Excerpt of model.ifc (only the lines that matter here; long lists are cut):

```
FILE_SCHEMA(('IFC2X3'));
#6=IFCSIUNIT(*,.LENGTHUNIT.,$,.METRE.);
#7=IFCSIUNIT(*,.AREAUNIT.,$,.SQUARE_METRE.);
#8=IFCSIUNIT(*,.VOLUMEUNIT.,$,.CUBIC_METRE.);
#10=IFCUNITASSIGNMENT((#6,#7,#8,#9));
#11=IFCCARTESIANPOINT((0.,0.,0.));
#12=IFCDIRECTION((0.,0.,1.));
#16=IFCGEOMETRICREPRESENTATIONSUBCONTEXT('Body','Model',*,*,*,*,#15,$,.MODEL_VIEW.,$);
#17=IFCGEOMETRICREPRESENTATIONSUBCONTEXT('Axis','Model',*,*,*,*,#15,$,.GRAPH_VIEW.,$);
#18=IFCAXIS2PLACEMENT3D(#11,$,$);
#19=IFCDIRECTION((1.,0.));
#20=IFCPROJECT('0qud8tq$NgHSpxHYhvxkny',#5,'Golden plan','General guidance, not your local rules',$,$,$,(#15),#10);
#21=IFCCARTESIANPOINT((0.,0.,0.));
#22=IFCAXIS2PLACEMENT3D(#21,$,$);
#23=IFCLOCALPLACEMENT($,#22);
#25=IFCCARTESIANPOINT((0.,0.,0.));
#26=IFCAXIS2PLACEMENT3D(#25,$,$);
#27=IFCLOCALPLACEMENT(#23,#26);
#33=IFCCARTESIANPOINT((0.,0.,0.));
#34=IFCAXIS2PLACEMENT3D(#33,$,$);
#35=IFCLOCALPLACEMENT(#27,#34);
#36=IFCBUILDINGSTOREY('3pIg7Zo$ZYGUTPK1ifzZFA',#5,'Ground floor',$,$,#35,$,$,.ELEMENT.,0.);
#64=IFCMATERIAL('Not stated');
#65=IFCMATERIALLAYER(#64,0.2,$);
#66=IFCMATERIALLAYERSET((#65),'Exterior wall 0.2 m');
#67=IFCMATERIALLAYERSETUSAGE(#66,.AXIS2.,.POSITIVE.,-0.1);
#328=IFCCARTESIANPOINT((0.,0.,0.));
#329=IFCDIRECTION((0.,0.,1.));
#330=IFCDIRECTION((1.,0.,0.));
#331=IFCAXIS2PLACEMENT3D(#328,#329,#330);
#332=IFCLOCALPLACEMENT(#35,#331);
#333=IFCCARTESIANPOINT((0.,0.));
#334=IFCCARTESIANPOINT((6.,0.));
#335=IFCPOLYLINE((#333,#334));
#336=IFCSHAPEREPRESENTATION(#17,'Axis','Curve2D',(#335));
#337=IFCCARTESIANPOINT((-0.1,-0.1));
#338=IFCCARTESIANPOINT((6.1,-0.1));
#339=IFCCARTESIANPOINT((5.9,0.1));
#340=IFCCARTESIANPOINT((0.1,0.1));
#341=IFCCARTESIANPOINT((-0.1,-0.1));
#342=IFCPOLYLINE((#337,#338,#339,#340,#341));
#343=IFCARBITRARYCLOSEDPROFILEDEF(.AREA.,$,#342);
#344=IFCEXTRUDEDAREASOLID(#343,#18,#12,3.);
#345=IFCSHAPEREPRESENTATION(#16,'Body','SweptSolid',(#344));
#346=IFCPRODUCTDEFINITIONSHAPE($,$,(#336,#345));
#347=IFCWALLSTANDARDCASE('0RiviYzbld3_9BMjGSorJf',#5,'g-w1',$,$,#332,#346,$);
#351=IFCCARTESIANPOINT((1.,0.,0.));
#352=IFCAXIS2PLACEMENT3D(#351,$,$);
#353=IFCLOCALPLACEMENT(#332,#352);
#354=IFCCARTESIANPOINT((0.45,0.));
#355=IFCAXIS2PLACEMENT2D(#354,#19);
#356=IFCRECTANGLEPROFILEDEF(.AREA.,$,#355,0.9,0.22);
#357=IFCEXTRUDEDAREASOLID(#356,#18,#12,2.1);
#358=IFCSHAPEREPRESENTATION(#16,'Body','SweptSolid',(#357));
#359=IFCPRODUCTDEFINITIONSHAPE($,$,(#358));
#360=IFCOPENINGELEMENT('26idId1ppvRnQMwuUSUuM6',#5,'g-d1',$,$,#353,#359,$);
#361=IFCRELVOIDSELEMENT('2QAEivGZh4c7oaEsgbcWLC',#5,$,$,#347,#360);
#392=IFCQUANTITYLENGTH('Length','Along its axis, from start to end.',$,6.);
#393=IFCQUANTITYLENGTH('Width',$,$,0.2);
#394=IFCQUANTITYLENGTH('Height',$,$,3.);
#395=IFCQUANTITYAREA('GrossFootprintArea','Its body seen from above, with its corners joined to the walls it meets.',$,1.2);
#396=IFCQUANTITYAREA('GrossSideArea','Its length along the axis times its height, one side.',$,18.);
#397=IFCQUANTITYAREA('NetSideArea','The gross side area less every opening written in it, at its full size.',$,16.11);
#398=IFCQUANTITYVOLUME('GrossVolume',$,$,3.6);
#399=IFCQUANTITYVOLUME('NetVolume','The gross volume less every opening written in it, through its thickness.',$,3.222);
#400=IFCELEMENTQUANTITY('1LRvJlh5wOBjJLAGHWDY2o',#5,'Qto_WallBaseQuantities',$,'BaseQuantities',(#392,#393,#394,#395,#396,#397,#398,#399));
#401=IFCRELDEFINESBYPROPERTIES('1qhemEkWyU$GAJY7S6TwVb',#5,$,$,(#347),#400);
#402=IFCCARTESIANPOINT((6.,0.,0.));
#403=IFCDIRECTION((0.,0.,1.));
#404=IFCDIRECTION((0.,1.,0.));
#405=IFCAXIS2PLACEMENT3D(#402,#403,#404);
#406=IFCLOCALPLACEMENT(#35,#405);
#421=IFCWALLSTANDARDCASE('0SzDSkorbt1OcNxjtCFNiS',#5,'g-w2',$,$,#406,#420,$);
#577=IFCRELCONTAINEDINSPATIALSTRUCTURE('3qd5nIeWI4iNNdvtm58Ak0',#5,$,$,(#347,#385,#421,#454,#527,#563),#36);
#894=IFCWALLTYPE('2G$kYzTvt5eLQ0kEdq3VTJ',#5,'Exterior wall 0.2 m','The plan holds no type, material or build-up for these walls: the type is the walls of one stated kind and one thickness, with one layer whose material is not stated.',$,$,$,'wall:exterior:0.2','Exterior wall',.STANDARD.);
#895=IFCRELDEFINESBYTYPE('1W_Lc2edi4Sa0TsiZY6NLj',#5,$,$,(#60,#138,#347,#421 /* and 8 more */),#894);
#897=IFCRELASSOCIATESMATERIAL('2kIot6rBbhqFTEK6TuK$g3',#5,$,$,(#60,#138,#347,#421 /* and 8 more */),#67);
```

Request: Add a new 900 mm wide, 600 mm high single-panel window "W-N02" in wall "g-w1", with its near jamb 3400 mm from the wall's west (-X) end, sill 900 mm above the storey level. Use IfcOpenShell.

```python
import numpy as np
import ifcopenshell
import ifcopenshell.api.feature
import ifcopenshell.api.geometry
import ifcopenshell.api.pset
import ifcopenshell.api.root
import ifcopenshell.api.spatial
import ifcopenshell.api.type
import ifcopenshell.geom
import ifcopenshell.util.element
import ifcopenshell.util.placement
import ifcopenshell.util.representation
import ifcopenshell.util.shape
import ifcopenshell.util.unit

model = ifcopenshell.open("model.ifc")
unit_scale = ifcopenshell.util.unit.calculate_unit_scale(model)
area_scale = ifcopenshell.util.unit.calculate_unit_scale(model, "AREAUNIT")
volume_scale = ifcopenshell.util.unit.calculate_unit_scale(model, "VOLUMEUNIT")
settings = ifcopenshell.geom.settings()


def volume(element):
    """Net volume in cubic metres, openings subtracted."""
    shape = ifcopenshell.geom.create_shape(settings, element)
    return ifcopenshell.util.shape.get_volume(shape.geometry)


wall = model.by_id(347)
storey = ifcopenshell.util.element.get_container(wall, ifc_class="IfcBuildingStorey")
context = ifcopenshell.util.representation.get_context(model, "Model", "Body", "MODEL_VIEW")
before = volume(wall)

width, height, from_end, sill = 0.9, 0.6, 3.4, 0.9  # metres

# The wall runs along its own X axis, and the end named is its -X end.
wall_shape = ifcopenshell.geom.create_shape(settings, wall)
x, y, z = ifcopenshell.util.shape.get_vertices(wall_shape.geometry).T
start = x.min() + from_end
face, thickness = float(y.min()), float(y.max() - y.min())
wall_matrix = ifcopenshell.util.placement.get_local_placement(wall.ObjectPlacement)
level = ifcopenshell.util.placement.get_local_placement(storey.ObjectPlacement)[2, 3]


def in_wall(x, y):
    """Placement at x, y metres in the wall's axes, at sill height."""
    matrix = wall_matrix.copy()
    matrix[:, 3] = wall_matrix @ np.array([x / unit_scale, y / unit_scale, 0.0, 1.0])
    matrix[2, 3] = level + sill / unit_scale
    return matrix


# Opening: a box that overshoots both wall faces by 50 mm.
opening = ifcopenshell.api.root.create_entity(model, ifc_class="IfcOpeningElement")
box = ifcopenshell.api.geometry.add_wall_representation(
    model, context=context, length=width, height=height, thickness=thickness + 0.1
)
ifcopenshell.api.geometry.assign_representation(model, product=opening, representation=box)
ifcopenshell.api.geometry.edit_object_placement(model, product=opening, matrix=in_wall(start, face - 0.05), is_si=False)
ifcopenshell.api.feature.add_feature(model, feature=opening, element=wall)

window = ifcopenshell.api.root.create_entity(model, ifc_class="IfcWindow", name="W-N02")
window.OverallWidth, window.OverallHeight = width / unit_scale, height / unit_scale
body = ifcopenshell.api.geometry.add_window_representation(
    model,
    context=context,
    overall_width=window.OverallWidth,
    overall_height=window.OverallHeight,
    partition_type="SINGLE_PANEL",
)
ifcopenshell.api.geometry.assign_representation(model, product=window, representation=body)
ifcopenshell.api.spatial.assign_container(model, products=[window], relating_structure=storey)
fills = ifcopenshell.api.feature.add_filling(model, opening=opening, element=window)
fills.OwnerHistory = window.OwnerHistory  # required in IFC2X3

# IFC2X3 keeps the operation on the window style.
style = ifcopenshell.api.root.create_entity(model, ifc_class="IfcWindowStyle", name="W-N02")
style.OperationType, style.ConstructionType = "SINGLE_PANEL", "NOTDEFINED"
style.ParameterTakesPrecedence = style.Sizeable = False
ifcopenshell.api.type.assign_type(model, related_objects=[window], relating_type=style)

# Centre the window in the wall's thickness.
ifcopenshell.api.geometry.edit_object_placement(model, product=window, matrix=in_wall(start, face), is_si=False)
window_shape = ifcopenshell.geom.create_shape(settings, window)
depth = ifcopenshell.util.shape.get_vertices(window_shape.geometry)[:, 1]
offset = face + thickness / 2 - (depth.min() + depth.max()) / 2
ifcopenshell.api.geometry.edit_object_placement(model, product=window, matrix=in_wall(start, offset), is_si=False)

after = volume(wall)

# Update the wall's stored quantities.
qto = model.by_id(ifcopenshell.util.element.get_pset(wall, "Qto_WallBaseQuantities", should_inherit=False)["id"])
ifcopenshell.api.pset.edit_qto(model, qto=qto, properties={
    "NetSideArea": after / thickness / area_scale,
    "NetVolume": after / volume_scale,
})

print(f"wall volume {before:.3f} -> {after:.3f} m3")

model.write("model_edited.ifc")
```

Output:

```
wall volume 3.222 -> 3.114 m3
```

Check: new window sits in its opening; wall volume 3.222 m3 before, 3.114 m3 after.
